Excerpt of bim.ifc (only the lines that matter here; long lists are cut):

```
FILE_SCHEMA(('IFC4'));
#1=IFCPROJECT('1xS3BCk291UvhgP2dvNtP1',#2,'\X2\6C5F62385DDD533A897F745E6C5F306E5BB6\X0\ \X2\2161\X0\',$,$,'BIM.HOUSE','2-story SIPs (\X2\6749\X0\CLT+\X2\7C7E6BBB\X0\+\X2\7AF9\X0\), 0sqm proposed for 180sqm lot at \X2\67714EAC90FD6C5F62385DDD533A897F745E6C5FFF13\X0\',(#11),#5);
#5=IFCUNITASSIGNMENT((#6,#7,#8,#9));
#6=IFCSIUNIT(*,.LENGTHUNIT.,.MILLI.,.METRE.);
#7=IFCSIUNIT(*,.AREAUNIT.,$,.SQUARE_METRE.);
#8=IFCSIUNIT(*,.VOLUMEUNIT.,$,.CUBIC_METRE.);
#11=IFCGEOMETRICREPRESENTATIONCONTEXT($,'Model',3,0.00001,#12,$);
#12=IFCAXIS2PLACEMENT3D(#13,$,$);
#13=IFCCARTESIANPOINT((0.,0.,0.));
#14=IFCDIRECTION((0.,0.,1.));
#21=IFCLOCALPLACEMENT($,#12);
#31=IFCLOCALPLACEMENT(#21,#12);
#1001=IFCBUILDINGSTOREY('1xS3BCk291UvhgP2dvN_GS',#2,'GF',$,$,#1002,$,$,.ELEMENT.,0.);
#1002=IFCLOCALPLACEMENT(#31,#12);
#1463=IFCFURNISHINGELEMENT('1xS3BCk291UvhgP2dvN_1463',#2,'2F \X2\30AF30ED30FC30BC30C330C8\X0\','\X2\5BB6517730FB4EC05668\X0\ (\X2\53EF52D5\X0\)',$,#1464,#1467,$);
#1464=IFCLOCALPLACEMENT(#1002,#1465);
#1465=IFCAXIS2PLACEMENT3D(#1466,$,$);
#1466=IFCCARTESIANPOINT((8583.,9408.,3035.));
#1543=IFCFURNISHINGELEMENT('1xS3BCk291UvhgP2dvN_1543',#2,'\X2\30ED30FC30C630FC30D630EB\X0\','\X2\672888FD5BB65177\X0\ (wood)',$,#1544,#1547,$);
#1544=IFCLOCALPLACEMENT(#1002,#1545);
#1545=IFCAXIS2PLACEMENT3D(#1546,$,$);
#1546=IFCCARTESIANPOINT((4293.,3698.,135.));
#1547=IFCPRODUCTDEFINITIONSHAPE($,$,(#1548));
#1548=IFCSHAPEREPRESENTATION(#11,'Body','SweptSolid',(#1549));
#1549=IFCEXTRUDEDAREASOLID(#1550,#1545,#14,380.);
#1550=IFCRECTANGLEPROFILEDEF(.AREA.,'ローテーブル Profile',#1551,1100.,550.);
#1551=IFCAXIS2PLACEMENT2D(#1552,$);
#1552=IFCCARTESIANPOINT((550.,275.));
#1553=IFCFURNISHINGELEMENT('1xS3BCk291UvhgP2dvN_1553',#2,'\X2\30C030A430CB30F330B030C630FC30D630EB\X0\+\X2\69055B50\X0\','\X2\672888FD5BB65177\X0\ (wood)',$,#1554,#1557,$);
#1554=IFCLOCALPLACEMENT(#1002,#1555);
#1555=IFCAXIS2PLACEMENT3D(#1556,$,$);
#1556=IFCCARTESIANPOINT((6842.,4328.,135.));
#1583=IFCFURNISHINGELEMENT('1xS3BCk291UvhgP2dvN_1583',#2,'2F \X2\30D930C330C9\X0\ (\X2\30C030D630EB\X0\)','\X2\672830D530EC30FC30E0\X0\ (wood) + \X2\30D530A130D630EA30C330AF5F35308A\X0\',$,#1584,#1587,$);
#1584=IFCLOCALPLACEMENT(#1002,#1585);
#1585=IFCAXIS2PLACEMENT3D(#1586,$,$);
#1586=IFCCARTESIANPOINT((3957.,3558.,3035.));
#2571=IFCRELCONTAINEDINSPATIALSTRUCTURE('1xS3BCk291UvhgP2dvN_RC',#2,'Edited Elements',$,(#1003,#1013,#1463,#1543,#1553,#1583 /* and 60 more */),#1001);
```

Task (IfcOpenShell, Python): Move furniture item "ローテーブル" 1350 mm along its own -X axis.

```python
import ifcopenshell
import ifcopenshell.api.geometry
import ifcopenshell.util.placement

model = ifcopenshell.open("bim.ifc")

item = model.by_guid("1xS3BCk291UvhgP2dvN_1543")
matrix = ifcopenshell.util.placement.get_local_placement(item.ObjectPlacement)
matrix[:3, 3] -= matrix[:3, 0] * 1350.0
ifcopenshell.api.geometry.edit_object_placement(model, product=item, matrix=matrix, is_si=False)

print(ifcopenshell.util.placement.get_local_placement(item.ObjectPlacement).round(3) + 0.0)

model.write("bim_edited.ifc")
```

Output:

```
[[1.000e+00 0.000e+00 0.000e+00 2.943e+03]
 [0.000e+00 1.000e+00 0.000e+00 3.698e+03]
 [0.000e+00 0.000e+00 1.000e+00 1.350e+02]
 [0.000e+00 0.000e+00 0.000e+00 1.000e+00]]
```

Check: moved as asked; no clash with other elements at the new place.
